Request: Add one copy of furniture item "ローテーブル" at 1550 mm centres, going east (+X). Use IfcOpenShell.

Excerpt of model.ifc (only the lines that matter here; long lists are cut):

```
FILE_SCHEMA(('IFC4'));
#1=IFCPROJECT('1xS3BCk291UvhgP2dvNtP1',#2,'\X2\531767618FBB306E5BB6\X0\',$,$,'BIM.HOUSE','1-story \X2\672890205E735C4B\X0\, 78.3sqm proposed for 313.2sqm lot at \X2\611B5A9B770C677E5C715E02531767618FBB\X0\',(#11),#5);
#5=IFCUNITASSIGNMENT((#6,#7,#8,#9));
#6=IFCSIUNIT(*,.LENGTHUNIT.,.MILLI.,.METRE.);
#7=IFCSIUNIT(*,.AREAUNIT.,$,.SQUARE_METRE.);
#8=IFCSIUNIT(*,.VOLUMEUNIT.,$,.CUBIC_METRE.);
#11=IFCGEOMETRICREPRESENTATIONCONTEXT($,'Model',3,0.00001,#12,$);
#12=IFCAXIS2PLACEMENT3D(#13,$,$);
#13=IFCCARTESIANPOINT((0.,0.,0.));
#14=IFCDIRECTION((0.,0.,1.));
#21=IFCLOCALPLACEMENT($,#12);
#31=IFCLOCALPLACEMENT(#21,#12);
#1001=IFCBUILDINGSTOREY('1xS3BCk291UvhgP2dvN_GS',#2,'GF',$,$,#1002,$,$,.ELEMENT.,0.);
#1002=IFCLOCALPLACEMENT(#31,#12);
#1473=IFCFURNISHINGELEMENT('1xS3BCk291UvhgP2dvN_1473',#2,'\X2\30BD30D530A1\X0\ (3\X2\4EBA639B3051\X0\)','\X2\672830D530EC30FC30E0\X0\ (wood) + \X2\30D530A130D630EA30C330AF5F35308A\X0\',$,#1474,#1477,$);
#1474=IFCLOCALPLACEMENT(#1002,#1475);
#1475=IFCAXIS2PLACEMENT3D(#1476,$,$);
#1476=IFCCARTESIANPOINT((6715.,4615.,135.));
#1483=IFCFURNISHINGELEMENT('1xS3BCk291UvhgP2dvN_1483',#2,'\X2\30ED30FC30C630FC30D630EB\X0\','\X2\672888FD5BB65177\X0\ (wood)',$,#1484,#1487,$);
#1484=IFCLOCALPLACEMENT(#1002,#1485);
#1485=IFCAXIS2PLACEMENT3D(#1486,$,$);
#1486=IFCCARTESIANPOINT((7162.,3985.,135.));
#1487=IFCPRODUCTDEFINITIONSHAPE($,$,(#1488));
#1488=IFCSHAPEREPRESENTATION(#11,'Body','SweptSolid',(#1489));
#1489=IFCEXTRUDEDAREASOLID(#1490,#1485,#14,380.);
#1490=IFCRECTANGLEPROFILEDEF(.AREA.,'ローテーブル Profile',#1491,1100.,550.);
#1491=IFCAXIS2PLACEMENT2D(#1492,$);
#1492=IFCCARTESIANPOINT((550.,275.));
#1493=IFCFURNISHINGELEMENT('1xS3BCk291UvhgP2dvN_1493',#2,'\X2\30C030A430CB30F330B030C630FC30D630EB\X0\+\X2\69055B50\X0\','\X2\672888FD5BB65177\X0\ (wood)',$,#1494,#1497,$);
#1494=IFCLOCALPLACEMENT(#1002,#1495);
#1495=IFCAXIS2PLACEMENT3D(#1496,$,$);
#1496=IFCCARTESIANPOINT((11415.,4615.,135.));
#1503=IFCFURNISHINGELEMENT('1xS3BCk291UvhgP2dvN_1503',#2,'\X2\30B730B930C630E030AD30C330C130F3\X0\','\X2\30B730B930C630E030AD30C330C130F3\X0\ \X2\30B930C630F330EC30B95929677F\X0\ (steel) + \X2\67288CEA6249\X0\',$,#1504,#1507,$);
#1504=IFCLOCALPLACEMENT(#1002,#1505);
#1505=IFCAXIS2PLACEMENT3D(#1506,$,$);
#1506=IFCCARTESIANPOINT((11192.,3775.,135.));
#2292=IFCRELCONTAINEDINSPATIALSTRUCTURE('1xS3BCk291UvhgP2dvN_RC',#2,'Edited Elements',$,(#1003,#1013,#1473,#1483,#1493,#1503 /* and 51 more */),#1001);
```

```python
import numpy as np
import ifcopenshell
import ifcopenshell.api.geometry
import ifcopenshell.api.root
import ifcopenshell.util.element
import ifcopenshell.util.placement
import ifcopenshell.util.unit

model = ifcopenshell.open("model.ifc")
unit_scale = ifcopenshell.util.unit.calculate_unit_scale(model)


def reuse_history(source, copy):
    """copy_class also copies each property set's owner history, people and application; keep the originals."""
    for rel in copy.IsDefinedBy:
        if rel.is_a("IfcRelDefinesByProperties") and (history := rel.RelatingPropertyDefinition.OwnerHistory):
            rel.RelatingPropertyDefinition.OwnerHistory = source.OwnerHistory
            ifcopenshell.util.element.remove_deep2(model, history)


source = model.by_guid("1xS3BCk291UvhgP2dvN_1483")
base = ifcopenshell.util.placement.get_local_placement(source.ObjectPlacement)
step = np.array([1.0, 0.0, 0.0]) * 1.55 / unit_scale

for i in range(1, 2):
    copy = ifcopenshell.api.root.copy_class(model, product=source)
    copy.Representation = ifcopenshell.util.element.copy_deep(
        model, source.Representation, exclude=["IfcGeometricRepresentationContext", "IfcRepresentationMap"]
    )
    reuse_history(source, copy)
    matrix = base.copy()
    matrix[:3, 3] += i * step
    print("added at", matrix[:3, 3].round(3) + 0.0)
    ifcopenshell.api.geometry.edit_object_placement(model, product=copy, matrix=matrix, is_si=False)

model.write("model-out.ifc")
```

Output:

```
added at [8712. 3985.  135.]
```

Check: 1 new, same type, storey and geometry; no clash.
